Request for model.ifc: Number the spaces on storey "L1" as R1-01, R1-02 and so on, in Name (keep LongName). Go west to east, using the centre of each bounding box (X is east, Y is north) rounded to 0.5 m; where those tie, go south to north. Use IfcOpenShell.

First a look at what the model holds.

```python
import ifcopenshell
import ifcopenshell.util.element
import ifcopenshell.util.placement

model = ifcopenshell.open("model.ifc")
print(model.schema)
storey = next(s for s in model.by_type("IfcBuildingStorey") if s.Name == "L1")
spaces = [e for e in ifcopenshell.util.element.get_decomposition(storey) if e.is_a("IfcSpace")]
for e in sorted(spaces, key=lambda e: e.id()):
    origin = ifcopenshell.util.placement.get_local_placement(e.ObjectPlacement)[:3, 3]
    print(e.id(), e.Name, e.LongName, origin.round(2) + 0.0, sep=" | ")
```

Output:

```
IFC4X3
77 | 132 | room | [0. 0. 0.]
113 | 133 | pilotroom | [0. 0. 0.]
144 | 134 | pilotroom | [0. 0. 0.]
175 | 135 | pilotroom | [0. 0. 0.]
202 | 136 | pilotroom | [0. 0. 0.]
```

```python
import ifcopenshell
import ifcopenshell.geom
import ifcopenshell.util.element
import ifcopenshell.util.shape

model = ifcopenshell.open("model.ifc")
settings = ifcopenshell.geom.settings()
settings.set("use-world-coords", True)


def centre(element):
    shape = ifcopenshell.geom.create_shape(settings, element)
    return ifcopenshell.util.shape.get_bbox_centroid(shape.geometry)


storey = next(s for s in model.by_type("IfcBuildingStorey") if s.Name == "L1")
spaces = [e for e in ifcopenshell.util.element.get_decomposition(storey) if e.is_a("IfcSpace")]

# Insertion points can sit at a corner or the storey origin, so sort by the geometry (in metres).
centres = {e: centre(e) for e in spaces}
spaces.sort(key=lambda e: (round(centres[e][0] / 0.5), centres[e][1]))

for i, e in enumerate(spaces, start=1):
    number = f"R1-{i:02d}"
    e.Name = number
    print(e.id(), number)

model.write("model-out.ifc")
```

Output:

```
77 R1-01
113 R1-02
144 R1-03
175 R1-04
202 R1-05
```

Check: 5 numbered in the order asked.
